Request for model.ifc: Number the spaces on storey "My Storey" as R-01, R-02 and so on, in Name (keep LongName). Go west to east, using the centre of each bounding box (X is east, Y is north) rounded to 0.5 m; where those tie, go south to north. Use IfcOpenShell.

First a look at what the model holds.

```python
import ifcopenshell
import ifcopenshell.util.element
import ifcopenshell.util.placement

model = ifcopenshell.open("model.ifc")
print(model.schema)
storey = next(s for s in model.by_type("IfcBuildingStorey") if s.Name == "My Storey")
spaces = [e for e in ifcopenshell.util.element.get_decomposition(storey) if e.is_a("IfcSpace")]
for e in sorted(spaces, key=lambda e: e.id()):
    origin = ifcopenshell.util.placement.get_local_placement(e.ObjectPlacement)[:3, 3]
    print(e.id(), e.Name, e.LongName, origin.round(2) + 0.0, sep=" | ")
```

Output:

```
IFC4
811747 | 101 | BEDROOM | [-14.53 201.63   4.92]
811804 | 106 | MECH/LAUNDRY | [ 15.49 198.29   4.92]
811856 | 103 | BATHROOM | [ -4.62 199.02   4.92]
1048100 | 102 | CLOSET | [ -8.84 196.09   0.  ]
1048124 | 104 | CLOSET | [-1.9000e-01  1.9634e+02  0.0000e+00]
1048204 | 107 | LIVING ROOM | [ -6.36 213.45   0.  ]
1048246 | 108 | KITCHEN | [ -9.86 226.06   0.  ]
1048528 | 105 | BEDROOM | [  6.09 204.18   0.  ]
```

```python
import ifcopenshell
import ifcopenshell.geom
import ifcopenshell.util.element
import ifcopenshell.util.shape

model = ifcopenshell.open("model.ifc")
settings = ifcopenshell.geom.settings()
settings.set("use-world-coords", True)


def centre(element):
    shape = ifcopenshell.geom.create_shape(settings, element)
    return ifcopenshell.util.shape.get_bbox_centroid(shape.geometry)


storey = next(s for s in model.by_type("IfcBuildingStorey") if s.Name == "My Storey")
spaces = [e for e in ifcopenshell.util.element.get_decomposition(storey) if e.is_a("IfcSpace")]

# Insertion points can sit at a corner or the storey origin, so sort by the geometry (in metres).
centres = {e: centre(e) for e in spaces}
spaces.sort(key=lambda e: (round(centres[e][0] / 0.5), centres[e][1]))

for i, e in enumerate(spaces, start=1):
    number = f"R-{i:02d}"
    e.Name = number
    print(e.id(), number)

model.write("model_edited.ifc")
```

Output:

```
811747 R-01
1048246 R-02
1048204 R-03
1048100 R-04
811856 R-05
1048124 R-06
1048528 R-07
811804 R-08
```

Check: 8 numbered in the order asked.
